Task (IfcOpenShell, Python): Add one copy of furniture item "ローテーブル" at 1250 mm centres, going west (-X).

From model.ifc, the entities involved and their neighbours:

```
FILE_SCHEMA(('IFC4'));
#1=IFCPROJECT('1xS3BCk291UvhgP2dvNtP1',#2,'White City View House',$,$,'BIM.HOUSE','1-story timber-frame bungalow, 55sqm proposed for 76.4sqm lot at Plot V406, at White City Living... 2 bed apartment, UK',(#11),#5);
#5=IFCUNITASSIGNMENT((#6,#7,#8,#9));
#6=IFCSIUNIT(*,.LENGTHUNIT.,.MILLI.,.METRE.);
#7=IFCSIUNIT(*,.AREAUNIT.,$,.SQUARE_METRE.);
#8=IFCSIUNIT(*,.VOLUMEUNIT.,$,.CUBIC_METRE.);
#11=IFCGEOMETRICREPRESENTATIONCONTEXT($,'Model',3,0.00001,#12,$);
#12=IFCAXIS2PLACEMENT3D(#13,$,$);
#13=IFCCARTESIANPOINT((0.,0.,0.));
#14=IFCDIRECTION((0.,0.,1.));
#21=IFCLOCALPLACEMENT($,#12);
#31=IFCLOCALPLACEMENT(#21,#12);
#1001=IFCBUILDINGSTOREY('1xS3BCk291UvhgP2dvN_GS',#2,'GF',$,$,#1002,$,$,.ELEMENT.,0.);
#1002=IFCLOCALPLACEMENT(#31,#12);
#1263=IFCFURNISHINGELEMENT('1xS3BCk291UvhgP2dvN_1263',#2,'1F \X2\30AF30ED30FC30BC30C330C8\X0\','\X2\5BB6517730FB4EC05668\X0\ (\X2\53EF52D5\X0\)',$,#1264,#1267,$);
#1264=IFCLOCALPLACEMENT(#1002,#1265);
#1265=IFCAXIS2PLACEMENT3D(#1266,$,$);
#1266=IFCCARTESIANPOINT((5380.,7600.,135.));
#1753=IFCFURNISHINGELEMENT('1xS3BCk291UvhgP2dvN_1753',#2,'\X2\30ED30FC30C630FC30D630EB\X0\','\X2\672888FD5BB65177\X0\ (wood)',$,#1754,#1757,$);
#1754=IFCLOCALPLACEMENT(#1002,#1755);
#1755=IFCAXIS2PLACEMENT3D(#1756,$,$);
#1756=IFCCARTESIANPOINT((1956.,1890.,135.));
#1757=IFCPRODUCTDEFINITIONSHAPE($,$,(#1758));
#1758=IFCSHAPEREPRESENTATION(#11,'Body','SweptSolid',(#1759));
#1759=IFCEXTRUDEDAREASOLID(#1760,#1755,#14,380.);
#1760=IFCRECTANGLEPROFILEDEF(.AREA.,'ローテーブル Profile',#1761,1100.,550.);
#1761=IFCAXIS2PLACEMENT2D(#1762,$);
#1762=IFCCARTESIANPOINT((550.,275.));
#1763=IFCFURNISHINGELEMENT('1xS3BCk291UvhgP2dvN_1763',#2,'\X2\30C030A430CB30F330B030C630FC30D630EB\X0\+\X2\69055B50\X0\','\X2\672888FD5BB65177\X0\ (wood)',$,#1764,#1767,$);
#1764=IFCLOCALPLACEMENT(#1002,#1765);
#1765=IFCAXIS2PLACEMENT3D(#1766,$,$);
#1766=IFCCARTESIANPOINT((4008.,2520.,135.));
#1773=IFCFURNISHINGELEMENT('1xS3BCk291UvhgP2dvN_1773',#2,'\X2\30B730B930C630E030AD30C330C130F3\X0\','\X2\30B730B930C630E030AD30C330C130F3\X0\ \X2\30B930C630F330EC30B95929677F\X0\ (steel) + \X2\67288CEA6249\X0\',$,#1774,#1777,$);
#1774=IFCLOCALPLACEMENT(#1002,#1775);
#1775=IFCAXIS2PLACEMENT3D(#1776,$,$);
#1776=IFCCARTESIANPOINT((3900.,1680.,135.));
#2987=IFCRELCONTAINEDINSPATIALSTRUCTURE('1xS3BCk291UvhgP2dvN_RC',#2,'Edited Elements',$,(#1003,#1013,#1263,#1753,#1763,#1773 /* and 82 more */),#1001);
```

```python
import numpy as np
import ifcopenshell
import ifcopenshell.api.geometry
import ifcopenshell.api.root
import ifcopenshell.util.element
import ifcopenshell.util.placement

model = ifcopenshell.open("model.ifc")


def reuse_history(source, copy):
    """copy_class also copies each property set's owner history, people and application; keep the originals."""
    for rel in copy.IsDefinedBy:
        if rel.is_a("IfcRelDefinesByProperties") and (history := rel.RelatingPropertyDefinition.OwnerHistory):
            rel.RelatingPropertyDefinition.OwnerHistory = source.OwnerHistory
            ifcopenshell.util.element.remove_deep2(model, history)


source = model.by_id(1753)
base = ifcopenshell.util.placement.get_local_placement(source.ObjectPlacement)
step = np.array([-1.0, 0.0, 0.0]) * 1250.0

for i in range(1, 2):
    copy = ifcopenshell.api.root.copy_class(model, product=source)
    copy.Representation = ifcopenshell.util.element.copy_deep(
        model, source.Representation, exclude=["IfcGeometricRepresentationContext", "IfcRepresentationMap"]
    )
    reuse_history(source, copy)
    matrix = base.copy()
    matrix[:3, 3] += i * step
    print("added at", matrix[:3, 3].round(3) + 0.0)
    ifcopenshell.api.geometry.edit_object_placement(model, product=copy, matrix=matrix, is_si=False)

model.write("model-out.ifc")
```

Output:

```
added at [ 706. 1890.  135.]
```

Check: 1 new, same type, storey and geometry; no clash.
